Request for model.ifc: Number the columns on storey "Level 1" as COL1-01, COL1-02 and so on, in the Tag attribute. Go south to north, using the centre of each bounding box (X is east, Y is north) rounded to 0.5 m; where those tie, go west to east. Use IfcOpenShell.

First a look at what the model holds.

```python
import ifcopenshell
import ifcopenshell.util.element
import ifcopenshell.util.placement

model = ifcopenshell.open("model.ifc")
print(model.schema)
storey = next(s for s in model.by_type("IfcBuildingStorey") if s.Name == "Level 1")
columns = [e for e in ifcopenshell.util.element.get_decomposition(storey) if e.is_a("IfcColumn")]
for e in sorted(columns, key=lambda e: e.id()):
    origin = ifcopenshell.util.placement.get_local_placement(e.ObjectPlacement)[:3, 3]
    print(e.id(), e.Tag, e.Name, origin.round(2) + 0.0, sep=" | ")
```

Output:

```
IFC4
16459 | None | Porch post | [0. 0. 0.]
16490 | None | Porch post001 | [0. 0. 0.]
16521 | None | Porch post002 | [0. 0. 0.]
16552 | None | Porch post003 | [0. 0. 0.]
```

```python
import ifcopenshell
import ifcopenshell.geom
import ifcopenshell.util.element
import ifcopenshell.util.shape

model = ifcopenshell.open("model.ifc")
settings = ifcopenshell.geom.settings()
settings.set("use-world-coords", True)


def centre(element):
    shape = ifcopenshell.geom.create_shape(settings, element)
    return ifcopenshell.util.shape.get_bbox_centroid(shape.geometry)


storey = next(s for s in model.by_type("IfcBuildingStorey") if s.Name == "Level 1")
columns = [e for e in ifcopenshell.util.element.get_decomposition(storey) if e.is_a("IfcColumn")]

# Insertion points can sit at a corner or the storey origin, so sort by the geometry (in metres).
centres = {e: centre(e) for e in columns}
columns.sort(key=lambda e: (round(centres[e][1] / 0.5), centres[e][0]))

for i, e in enumerate(columns, start=1):
    number = f"COL1-{i:02d}"
    e.Tag = number
    print(e.id(), number)

model.write("model_updated.ifc")
```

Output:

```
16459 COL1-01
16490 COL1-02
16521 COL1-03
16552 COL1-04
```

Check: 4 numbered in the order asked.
